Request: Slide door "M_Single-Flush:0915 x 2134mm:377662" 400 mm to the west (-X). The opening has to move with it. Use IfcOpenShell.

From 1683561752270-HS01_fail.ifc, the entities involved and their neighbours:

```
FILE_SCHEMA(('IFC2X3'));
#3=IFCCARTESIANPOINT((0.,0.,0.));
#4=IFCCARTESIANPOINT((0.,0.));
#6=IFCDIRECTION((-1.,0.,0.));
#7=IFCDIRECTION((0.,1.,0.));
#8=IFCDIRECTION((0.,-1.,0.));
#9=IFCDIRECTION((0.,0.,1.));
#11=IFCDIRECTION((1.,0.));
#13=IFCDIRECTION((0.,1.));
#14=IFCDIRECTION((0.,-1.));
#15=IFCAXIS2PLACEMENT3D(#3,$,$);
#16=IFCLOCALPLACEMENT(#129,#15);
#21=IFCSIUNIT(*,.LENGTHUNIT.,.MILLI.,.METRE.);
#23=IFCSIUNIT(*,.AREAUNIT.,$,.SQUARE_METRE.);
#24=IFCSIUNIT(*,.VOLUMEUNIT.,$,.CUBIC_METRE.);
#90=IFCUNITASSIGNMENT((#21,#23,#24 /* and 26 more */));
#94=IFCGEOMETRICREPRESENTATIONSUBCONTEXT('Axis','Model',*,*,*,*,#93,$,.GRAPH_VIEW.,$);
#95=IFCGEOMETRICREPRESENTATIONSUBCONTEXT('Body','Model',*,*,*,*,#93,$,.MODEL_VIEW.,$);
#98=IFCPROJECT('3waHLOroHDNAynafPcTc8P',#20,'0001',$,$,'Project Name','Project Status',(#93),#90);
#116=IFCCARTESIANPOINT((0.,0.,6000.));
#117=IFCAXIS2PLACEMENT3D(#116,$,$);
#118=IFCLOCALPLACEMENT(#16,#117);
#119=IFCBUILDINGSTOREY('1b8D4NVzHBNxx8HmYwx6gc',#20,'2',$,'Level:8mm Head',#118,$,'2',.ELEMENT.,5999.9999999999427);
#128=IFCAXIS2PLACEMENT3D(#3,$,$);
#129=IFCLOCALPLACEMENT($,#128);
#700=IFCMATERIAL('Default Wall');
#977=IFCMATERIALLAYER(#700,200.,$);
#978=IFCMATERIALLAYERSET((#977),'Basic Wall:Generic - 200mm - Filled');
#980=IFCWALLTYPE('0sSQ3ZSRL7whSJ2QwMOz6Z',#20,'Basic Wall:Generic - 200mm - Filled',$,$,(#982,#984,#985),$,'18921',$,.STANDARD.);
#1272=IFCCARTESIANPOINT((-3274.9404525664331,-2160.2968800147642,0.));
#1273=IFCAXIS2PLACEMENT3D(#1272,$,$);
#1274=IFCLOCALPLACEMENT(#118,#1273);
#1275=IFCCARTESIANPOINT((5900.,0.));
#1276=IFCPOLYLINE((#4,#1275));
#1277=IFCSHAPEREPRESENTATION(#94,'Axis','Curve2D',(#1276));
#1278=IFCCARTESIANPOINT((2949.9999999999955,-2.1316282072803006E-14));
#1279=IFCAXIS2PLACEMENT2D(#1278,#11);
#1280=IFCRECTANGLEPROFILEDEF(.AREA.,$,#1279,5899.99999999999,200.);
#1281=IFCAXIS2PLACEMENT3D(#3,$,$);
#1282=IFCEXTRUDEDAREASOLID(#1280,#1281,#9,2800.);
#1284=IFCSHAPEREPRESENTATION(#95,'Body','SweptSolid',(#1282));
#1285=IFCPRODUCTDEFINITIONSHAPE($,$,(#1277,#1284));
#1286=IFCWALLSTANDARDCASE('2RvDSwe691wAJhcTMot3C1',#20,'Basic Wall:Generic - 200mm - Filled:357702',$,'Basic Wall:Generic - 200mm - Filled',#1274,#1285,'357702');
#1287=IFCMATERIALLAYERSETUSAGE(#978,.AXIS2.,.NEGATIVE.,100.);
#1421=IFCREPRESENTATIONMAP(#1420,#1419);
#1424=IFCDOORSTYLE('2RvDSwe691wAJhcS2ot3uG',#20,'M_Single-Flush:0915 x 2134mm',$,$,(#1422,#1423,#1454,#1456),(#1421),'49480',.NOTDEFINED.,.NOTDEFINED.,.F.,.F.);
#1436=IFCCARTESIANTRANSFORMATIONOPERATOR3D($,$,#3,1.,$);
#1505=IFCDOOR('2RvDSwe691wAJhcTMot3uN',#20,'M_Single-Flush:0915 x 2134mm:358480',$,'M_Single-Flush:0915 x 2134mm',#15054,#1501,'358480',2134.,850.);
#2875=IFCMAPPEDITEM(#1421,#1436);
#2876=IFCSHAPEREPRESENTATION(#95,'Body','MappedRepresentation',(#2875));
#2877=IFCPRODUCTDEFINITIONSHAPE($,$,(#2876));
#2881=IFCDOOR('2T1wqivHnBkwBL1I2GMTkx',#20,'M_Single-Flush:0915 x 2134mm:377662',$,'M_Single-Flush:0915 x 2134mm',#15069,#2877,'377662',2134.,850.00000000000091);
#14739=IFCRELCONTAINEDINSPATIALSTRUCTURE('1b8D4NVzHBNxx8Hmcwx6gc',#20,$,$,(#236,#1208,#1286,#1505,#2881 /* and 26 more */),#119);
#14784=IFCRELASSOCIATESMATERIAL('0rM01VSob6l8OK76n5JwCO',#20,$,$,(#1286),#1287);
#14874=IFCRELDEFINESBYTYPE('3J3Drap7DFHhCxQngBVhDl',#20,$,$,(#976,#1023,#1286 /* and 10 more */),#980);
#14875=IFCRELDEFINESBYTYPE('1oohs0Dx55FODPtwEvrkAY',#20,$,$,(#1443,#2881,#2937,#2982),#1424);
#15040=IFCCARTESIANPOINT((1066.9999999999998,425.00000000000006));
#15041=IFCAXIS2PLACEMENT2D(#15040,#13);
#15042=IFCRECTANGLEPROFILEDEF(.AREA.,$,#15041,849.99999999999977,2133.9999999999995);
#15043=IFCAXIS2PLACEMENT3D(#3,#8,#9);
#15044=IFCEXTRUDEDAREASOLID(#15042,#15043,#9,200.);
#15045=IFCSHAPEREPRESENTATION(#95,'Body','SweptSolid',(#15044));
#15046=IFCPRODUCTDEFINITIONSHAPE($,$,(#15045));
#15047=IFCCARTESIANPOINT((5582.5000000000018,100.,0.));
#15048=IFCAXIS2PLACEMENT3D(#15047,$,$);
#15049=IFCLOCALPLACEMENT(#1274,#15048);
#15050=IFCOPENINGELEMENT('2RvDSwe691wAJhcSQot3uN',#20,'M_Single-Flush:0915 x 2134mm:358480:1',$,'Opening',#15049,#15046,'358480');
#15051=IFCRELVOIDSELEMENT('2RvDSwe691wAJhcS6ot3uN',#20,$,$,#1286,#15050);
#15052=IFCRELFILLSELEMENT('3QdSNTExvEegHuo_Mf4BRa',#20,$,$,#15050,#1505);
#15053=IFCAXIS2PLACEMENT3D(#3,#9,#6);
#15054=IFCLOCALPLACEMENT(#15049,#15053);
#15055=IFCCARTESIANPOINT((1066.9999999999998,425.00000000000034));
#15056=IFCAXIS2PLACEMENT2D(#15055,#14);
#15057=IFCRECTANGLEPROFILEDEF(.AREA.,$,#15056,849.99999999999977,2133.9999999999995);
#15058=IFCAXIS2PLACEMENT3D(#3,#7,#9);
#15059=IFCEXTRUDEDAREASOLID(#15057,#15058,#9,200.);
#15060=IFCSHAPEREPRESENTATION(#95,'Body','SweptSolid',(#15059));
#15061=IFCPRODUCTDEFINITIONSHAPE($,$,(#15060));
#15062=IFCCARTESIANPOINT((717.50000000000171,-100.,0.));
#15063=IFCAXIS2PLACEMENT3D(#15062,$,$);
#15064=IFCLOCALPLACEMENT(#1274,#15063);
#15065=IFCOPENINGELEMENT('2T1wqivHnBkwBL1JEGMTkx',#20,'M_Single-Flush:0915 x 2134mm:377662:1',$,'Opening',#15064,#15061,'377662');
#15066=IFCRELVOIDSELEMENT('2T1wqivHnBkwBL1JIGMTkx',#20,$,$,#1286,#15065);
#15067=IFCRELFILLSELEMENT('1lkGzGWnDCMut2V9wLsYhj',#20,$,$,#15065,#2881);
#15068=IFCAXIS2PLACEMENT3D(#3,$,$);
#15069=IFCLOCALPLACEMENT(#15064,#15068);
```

```python
import ifcopenshell
import ifcopenshell.api.geometry
import ifcopenshell.util.placement
import ifcopenshell.util.unit

model = ifcopenshell.open("1683561752270-HS01_fail.ifc")
unit_scale = ifcopenshell.util.unit.calculate_unit_scale(model)

door = model.by_guid("2T1wqivHnBkwBL1I2GMTkx")
opening = door.FillsVoids[0].RelatingOpeningElement
wall = opening.VoidsElements[0].RelatingBuildingElement

wall_matrix = ifcopenshell.util.placement.get_local_placement(wall.ObjectPlacement)
shift = wall_matrix[:3, 0] * -0.4 / unit_scale
before = ifcopenshell.util.placement.get_local_placement(door.ObjectPlacement)[:3, 3].copy()

# The door is placed relative to its opening, so it follows when the opening moves.
matrix = ifcopenshell.util.placement.get_local_placement(opening.ObjectPlacement)
matrix[:3, 3] += shift
ifcopenshell.api.geometry.edit_object_placement(
    model, product=opening, matrix=matrix, is_si=False, should_transform_children=True
)

after = ifcopenshell.util.placement.get_local_placement(door.ObjectPlacement)[:3, 3]
print("door moved by", (after - before).round(3) + 0.0)

model.write("1683561752270-HS01_fail-out.ifc")
```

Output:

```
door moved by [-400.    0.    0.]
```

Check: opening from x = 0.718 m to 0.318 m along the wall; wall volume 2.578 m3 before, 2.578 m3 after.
